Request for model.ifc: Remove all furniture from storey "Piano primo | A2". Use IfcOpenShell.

First a look at what the model holds.

```python
import ifcopenshell
import ifcopenshell.util.element

model = ifcopenshell.open("model.ifc")
print(model.schema)
storey = next(s for s in model.by_type("IfcBuildingStorey") if s.Name == "Piano primo | A2")
furniture = [e for e in ifcopenshell.util.element.get_decomposition(storey) if e.is_a("IfcFurnishingElement")]
seen = {}
for e in furniture:
    element_type = ifcopenshell.util.element.get_type(e)
    name = element_type.Name if element_type not in (None, e) else None
    seen[name] = seen.get(name, 0) + 1
for name, count in sorted(seen.items(), key=str):
    print(count, "x", name)
```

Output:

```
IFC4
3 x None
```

```python
import ifcopenshell
import ifcopenshell.api.root
import ifcopenshell.util.element

model = ifcopenshell.open("model.ifc")

storey = next(s for s in model.by_type("IfcBuildingStorey") if s.Name == "Piano primo | A2")
furniture = [e for e in ifcopenshell.util.element.get_decomposition(storey) if e.is_a("IfcFurnishingElement")]

for e in furniture:
    ifcopenshell.api.root.remove_product(model, product=e)
print(len(furniture), "removed")

model.write("model-out.ifc")
```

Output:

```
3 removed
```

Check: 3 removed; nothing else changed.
